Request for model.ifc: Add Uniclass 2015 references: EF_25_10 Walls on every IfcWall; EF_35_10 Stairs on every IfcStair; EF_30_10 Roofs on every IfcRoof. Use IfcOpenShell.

First a look at what the model holds.

```python
import ifcopenshell

model = ifcopenshell.open("model.ifc")
print(model.schema)
print("classifications:", [c.Name for c in model.by_type("IfcClassification")])
for ifc_class in ("IfcDoor", "IfcRoof", "IfcStair", "IfcWall", "IfcWindow"):
    print(ifc_class, len(model.by_type(ifc_class)))
```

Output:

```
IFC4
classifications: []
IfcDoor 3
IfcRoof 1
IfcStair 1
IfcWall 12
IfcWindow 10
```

```python
import ifcopenshell
import ifcopenshell.api.classification

model = ifcopenshell.open("model.ifc")

system = ifcopenshell.api.classification.add_classification(model, classification="Uniclass 2015")

codes = {
    "IfcWall": ("EF_25_10", "Walls"),
    "IfcStair": ("EF_35_10", "Stairs"),
    "IfcRoof": ("EF_30_10", "Roofs"),
}
for ifc_class, (code, name) in codes.items():
    products = model.by_type(ifc_class)
    ifcopenshell.api.classification.add_reference(
        model, products=products, classification=system, identification=code, name=name
    )
    print(code, len(products))

model.write("model-out.ifc")
```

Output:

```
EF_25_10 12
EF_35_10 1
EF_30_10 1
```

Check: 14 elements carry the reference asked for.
